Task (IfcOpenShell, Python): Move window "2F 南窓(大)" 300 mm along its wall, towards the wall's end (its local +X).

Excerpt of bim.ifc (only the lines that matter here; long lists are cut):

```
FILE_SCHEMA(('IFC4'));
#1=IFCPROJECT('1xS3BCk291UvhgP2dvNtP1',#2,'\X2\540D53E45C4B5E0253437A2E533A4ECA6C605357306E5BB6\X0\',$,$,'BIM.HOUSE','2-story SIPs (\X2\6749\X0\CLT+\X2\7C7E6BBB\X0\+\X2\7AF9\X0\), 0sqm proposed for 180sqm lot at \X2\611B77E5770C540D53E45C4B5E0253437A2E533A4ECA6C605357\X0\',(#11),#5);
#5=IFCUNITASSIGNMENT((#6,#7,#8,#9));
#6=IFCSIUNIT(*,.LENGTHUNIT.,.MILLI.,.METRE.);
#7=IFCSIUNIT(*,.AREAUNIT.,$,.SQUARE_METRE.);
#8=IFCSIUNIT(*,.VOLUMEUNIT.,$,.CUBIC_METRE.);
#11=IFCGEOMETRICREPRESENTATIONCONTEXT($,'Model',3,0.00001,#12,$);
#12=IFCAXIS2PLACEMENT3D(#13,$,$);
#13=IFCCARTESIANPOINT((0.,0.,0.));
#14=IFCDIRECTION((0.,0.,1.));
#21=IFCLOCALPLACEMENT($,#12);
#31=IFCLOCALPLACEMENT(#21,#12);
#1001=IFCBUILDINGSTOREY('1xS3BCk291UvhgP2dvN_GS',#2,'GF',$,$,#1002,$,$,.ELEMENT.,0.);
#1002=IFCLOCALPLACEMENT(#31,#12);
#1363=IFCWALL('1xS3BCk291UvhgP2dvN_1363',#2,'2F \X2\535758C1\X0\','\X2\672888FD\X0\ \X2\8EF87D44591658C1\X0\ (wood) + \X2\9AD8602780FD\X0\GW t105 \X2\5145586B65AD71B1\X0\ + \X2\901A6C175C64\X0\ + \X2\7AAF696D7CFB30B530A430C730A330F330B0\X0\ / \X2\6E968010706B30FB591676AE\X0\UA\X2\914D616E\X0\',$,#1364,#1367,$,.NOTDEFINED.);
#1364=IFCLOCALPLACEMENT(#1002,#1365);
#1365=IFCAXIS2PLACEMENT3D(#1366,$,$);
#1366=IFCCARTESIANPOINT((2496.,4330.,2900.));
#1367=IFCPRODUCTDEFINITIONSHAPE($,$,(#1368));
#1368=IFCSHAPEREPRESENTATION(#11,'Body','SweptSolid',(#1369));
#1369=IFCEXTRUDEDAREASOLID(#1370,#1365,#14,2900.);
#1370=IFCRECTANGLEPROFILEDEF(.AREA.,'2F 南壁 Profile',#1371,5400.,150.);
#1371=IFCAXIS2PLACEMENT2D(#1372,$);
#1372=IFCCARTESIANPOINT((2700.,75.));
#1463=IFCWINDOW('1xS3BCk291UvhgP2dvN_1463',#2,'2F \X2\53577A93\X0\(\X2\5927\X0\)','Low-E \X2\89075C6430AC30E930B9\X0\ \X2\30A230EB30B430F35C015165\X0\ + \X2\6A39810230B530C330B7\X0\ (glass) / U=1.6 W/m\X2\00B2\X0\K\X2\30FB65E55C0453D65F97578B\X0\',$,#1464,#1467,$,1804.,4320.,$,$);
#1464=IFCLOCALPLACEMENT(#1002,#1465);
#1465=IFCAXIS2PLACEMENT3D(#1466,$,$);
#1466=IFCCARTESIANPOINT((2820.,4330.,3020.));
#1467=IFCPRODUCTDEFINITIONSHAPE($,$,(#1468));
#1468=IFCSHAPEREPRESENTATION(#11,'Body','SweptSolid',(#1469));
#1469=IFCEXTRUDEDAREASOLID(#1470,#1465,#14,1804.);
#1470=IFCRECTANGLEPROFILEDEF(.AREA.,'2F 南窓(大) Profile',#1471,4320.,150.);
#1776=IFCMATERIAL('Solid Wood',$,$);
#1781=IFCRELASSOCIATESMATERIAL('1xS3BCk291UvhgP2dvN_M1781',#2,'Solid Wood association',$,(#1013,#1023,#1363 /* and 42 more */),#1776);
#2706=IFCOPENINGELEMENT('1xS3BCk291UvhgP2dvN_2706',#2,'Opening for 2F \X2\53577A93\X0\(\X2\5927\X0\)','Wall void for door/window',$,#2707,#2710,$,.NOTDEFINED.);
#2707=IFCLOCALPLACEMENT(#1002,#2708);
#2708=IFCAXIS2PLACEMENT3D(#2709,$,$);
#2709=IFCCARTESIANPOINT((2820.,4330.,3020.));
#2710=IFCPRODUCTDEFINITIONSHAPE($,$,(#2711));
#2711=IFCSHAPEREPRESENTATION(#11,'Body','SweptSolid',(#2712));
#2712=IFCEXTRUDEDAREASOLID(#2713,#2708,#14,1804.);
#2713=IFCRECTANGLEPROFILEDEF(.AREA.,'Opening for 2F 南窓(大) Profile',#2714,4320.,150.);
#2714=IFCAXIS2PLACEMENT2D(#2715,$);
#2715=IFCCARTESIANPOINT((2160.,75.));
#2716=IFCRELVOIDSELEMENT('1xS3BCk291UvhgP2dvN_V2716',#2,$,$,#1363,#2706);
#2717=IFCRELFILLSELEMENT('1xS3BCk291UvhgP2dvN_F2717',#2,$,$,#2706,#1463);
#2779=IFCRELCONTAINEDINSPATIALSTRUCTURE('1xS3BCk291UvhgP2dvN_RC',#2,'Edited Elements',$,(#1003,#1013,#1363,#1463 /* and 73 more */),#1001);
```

```python
import ifcopenshell
import ifcopenshell.api.geometry
import ifcopenshell.util.placement
import ifcopenshell.util.unit

model = ifcopenshell.open("bim.ifc")
unit_scale = ifcopenshell.util.unit.calculate_unit_scale(model)

window = model.by_guid("1xS3BCk291UvhgP2dvN_1463")
opening = window.FillsVoids[0].RelatingOpeningElement
wall = opening.VoidsElements[0].RelatingBuildingElement

wall_matrix = ifcopenshell.util.placement.get_local_placement(wall.ObjectPlacement)
shift = wall_matrix[:3, 0] * 0.3 / unit_scale
before = ifcopenshell.util.placement.get_local_placement(window.ObjectPlacement)[:3, 3].copy()

# The window is not placed relative to its opening, so move both.
for product in (opening, window):
    matrix = ifcopenshell.util.placement.get_local_placement(product.ObjectPlacement)
    matrix[:3, 3] += shift
    ifcopenshell.api.geometry.edit_object_placement(model, product=product, matrix=matrix, is_si=False)

after = ifcopenshell.util.placement.get_local_placement(window.ObjectPlacement)[:3, 3]
print("window moved by", (after - before).round(3) + 0.0)

model.write("bim_v2.ifc")
```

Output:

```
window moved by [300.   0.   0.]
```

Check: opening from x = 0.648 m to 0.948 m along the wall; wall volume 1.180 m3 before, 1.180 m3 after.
